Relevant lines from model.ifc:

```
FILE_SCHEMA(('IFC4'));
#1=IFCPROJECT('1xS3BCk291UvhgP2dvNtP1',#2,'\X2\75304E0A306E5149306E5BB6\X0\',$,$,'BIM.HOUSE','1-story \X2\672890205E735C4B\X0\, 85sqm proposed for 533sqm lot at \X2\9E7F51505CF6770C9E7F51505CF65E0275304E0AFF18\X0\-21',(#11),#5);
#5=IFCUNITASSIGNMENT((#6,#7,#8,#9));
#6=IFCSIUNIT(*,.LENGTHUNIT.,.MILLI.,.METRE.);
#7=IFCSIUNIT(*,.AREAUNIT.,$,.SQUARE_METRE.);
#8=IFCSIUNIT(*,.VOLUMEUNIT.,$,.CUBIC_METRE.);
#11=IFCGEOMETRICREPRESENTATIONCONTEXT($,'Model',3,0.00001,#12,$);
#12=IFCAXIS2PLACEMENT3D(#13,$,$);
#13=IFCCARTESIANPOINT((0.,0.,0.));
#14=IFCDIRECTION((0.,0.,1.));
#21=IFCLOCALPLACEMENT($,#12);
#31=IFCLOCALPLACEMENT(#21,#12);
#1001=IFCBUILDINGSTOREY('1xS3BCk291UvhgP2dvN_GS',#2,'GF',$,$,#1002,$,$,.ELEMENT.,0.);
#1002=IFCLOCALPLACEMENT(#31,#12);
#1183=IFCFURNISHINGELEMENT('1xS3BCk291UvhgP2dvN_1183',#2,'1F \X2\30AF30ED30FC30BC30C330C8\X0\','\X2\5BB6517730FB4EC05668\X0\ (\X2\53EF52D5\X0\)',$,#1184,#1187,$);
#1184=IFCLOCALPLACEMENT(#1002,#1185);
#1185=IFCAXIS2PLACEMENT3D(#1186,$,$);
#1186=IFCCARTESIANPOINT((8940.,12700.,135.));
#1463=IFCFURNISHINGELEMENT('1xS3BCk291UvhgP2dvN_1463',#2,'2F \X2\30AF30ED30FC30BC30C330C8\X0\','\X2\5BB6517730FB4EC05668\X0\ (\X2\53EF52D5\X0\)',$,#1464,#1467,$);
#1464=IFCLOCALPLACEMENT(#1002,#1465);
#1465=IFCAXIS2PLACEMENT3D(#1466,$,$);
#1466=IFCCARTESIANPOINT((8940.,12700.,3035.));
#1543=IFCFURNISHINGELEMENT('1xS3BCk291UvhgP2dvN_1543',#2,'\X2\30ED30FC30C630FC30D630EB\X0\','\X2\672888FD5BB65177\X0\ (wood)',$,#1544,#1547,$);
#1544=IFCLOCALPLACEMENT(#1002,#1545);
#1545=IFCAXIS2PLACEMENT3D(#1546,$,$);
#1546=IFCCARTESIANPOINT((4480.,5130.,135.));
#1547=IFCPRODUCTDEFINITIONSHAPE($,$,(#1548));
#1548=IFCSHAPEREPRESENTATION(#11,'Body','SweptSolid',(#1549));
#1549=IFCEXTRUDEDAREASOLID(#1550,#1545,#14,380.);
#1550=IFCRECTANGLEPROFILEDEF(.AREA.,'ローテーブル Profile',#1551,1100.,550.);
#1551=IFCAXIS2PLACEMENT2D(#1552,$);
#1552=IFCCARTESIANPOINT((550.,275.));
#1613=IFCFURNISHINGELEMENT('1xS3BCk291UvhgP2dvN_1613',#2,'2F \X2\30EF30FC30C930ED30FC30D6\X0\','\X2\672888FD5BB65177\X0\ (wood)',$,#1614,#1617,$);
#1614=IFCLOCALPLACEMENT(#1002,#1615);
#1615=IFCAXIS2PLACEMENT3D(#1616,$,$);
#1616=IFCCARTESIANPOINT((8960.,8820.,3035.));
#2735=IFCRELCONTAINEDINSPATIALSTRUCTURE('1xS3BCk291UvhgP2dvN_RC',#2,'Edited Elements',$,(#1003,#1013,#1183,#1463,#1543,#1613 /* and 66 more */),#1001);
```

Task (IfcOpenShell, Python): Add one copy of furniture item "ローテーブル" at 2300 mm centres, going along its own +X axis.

```python
import ifcopenshell
import ifcopenshell.api.geometry
import ifcopenshell.api.root
import ifcopenshell.util.element
import ifcopenshell.util.placement
import ifcopenshell.util.unit

model = ifcopenshell.open("model.ifc")
unit_scale = ifcopenshell.util.unit.calculate_unit_scale(model)


def reuse_history(source, copy):
    """copy_class also copies each property set's owner history, people and application; keep the originals."""
    for rel in copy.IsDefinedBy:
        if rel.is_a("IfcRelDefinesByProperties") and (history := rel.RelatingPropertyDefinition.OwnerHistory):
            rel.RelatingPropertyDefinition.OwnerHistory = source.OwnerHistory
            ifcopenshell.util.element.remove_deep2(model, history)


source = model.by_guid("1xS3BCk291UvhgP2dvN_1543")
base = ifcopenshell.util.placement.get_local_placement(source.ObjectPlacement)
step = base[:3, 0] * 2.3 / unit_scale

for i in range(1, 2):
    copy = ifcopenshell.api.root.copy_class(model, product=source)
    copy.Representation = ifcopenshell.util.element.copy_deep(
        model, source.Representation, exclude=["IfcGeometricRepresentationContext", "IfcRepresentationMap"]
    )
    reuse_history(source, copy)
    matrix = base.copy()
    matrix[:3, 3] += i * step
    print("added at", matrix[:3, 3].round(3) + 0.0)
    ifcopenshell.api.geometry.edit_object_placement(model, product=copy, matrix=matrix, is_si=False)

model.write("model-out.ifc")
```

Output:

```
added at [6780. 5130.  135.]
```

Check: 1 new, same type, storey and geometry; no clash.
